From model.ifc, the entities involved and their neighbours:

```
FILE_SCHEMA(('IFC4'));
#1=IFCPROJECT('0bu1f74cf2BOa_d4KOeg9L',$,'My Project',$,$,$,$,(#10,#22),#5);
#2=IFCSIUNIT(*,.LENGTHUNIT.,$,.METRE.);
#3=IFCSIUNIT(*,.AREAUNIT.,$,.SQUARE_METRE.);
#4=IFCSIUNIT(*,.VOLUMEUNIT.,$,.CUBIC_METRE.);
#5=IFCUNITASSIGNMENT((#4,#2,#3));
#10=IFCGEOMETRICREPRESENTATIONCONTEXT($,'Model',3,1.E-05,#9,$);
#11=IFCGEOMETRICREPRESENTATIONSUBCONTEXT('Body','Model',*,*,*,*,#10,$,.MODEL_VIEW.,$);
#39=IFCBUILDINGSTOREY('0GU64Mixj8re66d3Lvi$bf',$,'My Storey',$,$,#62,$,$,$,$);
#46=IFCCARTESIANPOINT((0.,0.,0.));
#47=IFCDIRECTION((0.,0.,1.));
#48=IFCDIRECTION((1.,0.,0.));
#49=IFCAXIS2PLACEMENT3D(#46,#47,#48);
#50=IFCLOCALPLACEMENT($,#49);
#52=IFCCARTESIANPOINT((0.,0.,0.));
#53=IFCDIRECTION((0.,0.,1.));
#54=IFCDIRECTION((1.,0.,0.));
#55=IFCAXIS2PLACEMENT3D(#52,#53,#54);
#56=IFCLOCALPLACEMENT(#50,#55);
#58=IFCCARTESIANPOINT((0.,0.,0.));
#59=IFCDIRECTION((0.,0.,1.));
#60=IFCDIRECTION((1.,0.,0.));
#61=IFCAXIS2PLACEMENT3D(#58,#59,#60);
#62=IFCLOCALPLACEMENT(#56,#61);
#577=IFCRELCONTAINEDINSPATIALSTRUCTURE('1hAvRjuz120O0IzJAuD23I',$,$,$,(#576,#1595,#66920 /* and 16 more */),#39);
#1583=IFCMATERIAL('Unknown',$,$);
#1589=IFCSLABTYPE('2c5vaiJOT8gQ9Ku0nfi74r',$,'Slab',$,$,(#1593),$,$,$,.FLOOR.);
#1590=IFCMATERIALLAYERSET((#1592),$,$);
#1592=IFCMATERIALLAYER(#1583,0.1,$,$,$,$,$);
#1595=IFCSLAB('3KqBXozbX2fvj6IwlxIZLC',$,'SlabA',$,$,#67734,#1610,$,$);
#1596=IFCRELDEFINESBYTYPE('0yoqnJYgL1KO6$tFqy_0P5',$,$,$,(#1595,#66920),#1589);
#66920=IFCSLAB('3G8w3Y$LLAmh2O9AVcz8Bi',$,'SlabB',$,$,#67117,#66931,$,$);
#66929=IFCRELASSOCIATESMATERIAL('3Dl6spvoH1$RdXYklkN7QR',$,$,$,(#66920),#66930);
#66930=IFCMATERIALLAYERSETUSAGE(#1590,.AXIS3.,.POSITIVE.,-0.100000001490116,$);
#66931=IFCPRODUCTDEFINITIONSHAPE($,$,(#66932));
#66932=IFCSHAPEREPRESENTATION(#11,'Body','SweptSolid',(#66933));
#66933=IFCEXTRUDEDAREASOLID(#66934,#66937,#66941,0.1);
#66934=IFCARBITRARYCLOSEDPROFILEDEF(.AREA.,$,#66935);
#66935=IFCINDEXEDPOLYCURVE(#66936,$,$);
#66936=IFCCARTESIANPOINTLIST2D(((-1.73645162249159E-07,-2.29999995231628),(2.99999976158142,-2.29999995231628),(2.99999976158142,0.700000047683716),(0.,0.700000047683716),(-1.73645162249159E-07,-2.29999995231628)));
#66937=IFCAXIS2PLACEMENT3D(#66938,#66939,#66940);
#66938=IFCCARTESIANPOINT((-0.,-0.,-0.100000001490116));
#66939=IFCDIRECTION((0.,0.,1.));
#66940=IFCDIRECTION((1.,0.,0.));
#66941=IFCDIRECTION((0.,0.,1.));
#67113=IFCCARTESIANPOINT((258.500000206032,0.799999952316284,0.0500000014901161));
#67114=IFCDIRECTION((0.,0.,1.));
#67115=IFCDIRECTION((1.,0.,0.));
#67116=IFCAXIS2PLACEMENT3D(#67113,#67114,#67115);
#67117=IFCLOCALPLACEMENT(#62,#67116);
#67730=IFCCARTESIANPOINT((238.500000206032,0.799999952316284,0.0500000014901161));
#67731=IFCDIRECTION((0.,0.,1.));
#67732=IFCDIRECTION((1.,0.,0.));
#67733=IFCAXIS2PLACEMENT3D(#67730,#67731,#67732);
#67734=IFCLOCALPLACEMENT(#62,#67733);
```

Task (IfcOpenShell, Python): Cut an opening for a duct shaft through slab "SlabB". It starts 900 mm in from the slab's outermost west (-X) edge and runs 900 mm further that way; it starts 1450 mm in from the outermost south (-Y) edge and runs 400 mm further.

```python
import numpy as np
import ifcopenshell
import ifcopenshell.api.feature
import ifcopenshell.api.geometry
import ifcopenshell.api.root
import ifcopenshell.geom
import ifcopenshell.util.placement
import ifcopenshell.util.representation
import ifcopenshell.util.shape
import ifcopenshell.util.unit

model = ifcopenshell.open("model.ifc")
unit_scale = ifcopenshell.util.unit.calculate_unit_scale(model)
settings = ifcopenshell.geom.settings()


def volume(element):
    """Net volume in cubic metres, openings subtracted."""
    shape = ifcopenshell.geom.create_shape(settings, element)
    return ifcopenshell.util.shape.get_volume(shape.geometry)


slab = model.by_guid("3G8w3Y$LLAmh2O9AVcz8Bi")
before = volume(slab)

# Extent in the slab's own axes, in metres. The edges named are its -X and -Y sides.
slab_shape = ifcopenshell.geom.create_shape(settings, slab)
vertices = ifcopenshell.util.shape.get_vertices(slab_shape.geometry)
x_min, y_min, bottom = vertices.min(axis=0)
top = vertices[:, 2].max()

opening = ifcopenshell.api.root.create_entity(model, ifc_class="IfcOpeningElement", name="Duct shaft opening", predefined_type="OPENING")
context = ifcopenshell.util.representation.get_context(model, "Model", "Body", "MODEL_VIEW")
width, depth = 0.9, 0.4
outline = [(0.0, 0.0), (width, 0.0), (width, depth), (0.0, depth), (0.0, 0.0)]
# Overshoot both faces by 50 mm so the cut is clean.
shape = ifcopenshell.api.geometry.add_slab_representation(
    model, context=context, depth=top - bottom + 0.1, polyline=outline
)
ifcopenshell.api.geometry.assign_representation(model, product=opening, representation=shape)

matrix = ifcopenshell.util.placement.get_local_placement(slab.ObjectPlacement)
matrix[:, 3] = matrix @ np.append(np.array([x_min + 0.9, y_min + 1.45, bottom - 0.05]) / unit_scale, 1.0)
ifcopenshell.api.geometry.edit_object_placement(model, product=opening, matrix=matrix, is_si=False)
ifcopenshell.api.feature.add_feature(model, feature=opening, element=slab)

after = volume(slab)

print(f"slab volume {before:.3f} -> {after:.3f} m3")

model.write("model_edited.ifc")
```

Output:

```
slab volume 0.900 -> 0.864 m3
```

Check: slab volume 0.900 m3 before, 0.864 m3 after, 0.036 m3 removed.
